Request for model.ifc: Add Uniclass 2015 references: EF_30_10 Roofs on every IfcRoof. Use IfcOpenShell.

First a look at what the model holds.

```python
import ifcopenshell

model = ifcopenshell.open("model.ifc")
print(model.schema)
print("classifications:", [c.Name for c in model.by_type("IfcClassification")])
for ifc_class in ("IfcDoor", "IfcRoof", "IfcStair", "IfcWall", "IfcWindow"):
    print(ifc_class, len(model.by_type(ifc_class)))
```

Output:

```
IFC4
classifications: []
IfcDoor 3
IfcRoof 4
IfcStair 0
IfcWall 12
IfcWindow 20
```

```python
import ifcopenshell
import ifcopenshell.api.classification

model = ifcopenshell.open("model.ifc")

system = ifcopenshell.api.classification.add_classification(model, classification="Uniclass 2015")

codes = {
    "IfcRoof": ("EF_30_10", "Roofs"),
}
for ifc_class, (code, name) in codes.items():
    products = model.by_type(ifc_class)
    ifcopenshell.api.classification.add_reference(
        model, products=products, classification=system, identification=code, name=name
    )
    print(code, len(products))

model.write("model_v2.ifc")
```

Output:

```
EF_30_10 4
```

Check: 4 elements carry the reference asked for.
